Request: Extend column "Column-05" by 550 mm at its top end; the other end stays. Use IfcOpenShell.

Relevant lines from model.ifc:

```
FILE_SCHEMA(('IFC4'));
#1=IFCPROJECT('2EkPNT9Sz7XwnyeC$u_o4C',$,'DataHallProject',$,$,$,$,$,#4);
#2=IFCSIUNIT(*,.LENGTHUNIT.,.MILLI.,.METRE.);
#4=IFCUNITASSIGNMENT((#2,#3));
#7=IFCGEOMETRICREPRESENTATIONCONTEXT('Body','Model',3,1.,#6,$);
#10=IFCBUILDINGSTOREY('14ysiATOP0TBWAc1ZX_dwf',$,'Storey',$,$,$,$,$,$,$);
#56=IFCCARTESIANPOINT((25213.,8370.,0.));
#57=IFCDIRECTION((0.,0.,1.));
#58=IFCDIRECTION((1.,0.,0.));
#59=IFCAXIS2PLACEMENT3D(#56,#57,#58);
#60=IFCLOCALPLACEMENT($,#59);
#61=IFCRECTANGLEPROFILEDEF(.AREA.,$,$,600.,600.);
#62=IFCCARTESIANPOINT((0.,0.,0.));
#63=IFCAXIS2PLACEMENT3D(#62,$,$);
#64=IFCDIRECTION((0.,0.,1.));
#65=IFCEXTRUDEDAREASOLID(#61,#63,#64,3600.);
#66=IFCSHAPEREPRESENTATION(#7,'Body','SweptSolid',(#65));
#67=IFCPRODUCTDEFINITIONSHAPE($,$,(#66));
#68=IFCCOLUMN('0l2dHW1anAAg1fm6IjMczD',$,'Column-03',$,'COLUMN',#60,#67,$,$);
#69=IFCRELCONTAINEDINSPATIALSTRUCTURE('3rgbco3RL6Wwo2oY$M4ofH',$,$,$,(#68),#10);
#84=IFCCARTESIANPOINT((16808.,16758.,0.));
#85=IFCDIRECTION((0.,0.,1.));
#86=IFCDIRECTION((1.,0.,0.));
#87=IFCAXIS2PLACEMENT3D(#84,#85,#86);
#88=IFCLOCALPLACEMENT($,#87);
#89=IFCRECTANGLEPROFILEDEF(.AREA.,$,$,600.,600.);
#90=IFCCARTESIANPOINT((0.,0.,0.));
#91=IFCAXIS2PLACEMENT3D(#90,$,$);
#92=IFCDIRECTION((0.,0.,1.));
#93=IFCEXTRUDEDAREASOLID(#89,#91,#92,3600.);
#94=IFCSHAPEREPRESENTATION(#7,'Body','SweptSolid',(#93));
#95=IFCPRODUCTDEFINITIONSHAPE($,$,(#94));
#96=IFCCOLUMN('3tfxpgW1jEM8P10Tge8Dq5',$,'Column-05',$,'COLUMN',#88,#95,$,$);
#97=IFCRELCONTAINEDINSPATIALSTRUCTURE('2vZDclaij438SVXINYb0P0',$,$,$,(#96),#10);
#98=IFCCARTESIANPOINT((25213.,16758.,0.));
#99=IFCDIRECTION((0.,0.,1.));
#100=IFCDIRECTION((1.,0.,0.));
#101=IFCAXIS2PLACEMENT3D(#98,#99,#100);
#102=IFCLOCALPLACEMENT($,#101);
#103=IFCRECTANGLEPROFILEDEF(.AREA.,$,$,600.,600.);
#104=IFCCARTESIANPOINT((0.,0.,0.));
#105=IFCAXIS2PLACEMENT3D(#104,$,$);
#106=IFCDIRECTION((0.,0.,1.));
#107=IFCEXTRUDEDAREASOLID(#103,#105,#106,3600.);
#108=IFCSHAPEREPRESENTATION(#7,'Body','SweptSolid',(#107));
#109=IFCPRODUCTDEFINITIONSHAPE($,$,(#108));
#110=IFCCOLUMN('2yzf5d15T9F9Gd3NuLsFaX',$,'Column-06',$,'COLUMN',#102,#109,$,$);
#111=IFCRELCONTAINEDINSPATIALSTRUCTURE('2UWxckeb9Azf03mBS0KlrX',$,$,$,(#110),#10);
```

```python
import ifcopenshell
import ifcopenshell.util.unit

model = ifcopenshell.open("model.ifc")
unit_scale = ifcopenshell.util.unit.calculate_unit_scale(model)

member = model.by_guid("3tfxpgW1jEM8P10Tge8Dq5")
change = 0.55 / unit_scale

# The extrusion runs towards the end named, so only its depth changes.
body = next(r for r in member.Representation.Representations if r.RepresentationIdentifier == "Body")
solid = body.Items[0]
old_length = solid.Depth
solid.Depth += change

print(f"length {old_length:g} -> {solid.Depth:g}")

model.write("model_rev.ifc")
```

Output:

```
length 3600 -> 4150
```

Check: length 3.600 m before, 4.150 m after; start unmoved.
